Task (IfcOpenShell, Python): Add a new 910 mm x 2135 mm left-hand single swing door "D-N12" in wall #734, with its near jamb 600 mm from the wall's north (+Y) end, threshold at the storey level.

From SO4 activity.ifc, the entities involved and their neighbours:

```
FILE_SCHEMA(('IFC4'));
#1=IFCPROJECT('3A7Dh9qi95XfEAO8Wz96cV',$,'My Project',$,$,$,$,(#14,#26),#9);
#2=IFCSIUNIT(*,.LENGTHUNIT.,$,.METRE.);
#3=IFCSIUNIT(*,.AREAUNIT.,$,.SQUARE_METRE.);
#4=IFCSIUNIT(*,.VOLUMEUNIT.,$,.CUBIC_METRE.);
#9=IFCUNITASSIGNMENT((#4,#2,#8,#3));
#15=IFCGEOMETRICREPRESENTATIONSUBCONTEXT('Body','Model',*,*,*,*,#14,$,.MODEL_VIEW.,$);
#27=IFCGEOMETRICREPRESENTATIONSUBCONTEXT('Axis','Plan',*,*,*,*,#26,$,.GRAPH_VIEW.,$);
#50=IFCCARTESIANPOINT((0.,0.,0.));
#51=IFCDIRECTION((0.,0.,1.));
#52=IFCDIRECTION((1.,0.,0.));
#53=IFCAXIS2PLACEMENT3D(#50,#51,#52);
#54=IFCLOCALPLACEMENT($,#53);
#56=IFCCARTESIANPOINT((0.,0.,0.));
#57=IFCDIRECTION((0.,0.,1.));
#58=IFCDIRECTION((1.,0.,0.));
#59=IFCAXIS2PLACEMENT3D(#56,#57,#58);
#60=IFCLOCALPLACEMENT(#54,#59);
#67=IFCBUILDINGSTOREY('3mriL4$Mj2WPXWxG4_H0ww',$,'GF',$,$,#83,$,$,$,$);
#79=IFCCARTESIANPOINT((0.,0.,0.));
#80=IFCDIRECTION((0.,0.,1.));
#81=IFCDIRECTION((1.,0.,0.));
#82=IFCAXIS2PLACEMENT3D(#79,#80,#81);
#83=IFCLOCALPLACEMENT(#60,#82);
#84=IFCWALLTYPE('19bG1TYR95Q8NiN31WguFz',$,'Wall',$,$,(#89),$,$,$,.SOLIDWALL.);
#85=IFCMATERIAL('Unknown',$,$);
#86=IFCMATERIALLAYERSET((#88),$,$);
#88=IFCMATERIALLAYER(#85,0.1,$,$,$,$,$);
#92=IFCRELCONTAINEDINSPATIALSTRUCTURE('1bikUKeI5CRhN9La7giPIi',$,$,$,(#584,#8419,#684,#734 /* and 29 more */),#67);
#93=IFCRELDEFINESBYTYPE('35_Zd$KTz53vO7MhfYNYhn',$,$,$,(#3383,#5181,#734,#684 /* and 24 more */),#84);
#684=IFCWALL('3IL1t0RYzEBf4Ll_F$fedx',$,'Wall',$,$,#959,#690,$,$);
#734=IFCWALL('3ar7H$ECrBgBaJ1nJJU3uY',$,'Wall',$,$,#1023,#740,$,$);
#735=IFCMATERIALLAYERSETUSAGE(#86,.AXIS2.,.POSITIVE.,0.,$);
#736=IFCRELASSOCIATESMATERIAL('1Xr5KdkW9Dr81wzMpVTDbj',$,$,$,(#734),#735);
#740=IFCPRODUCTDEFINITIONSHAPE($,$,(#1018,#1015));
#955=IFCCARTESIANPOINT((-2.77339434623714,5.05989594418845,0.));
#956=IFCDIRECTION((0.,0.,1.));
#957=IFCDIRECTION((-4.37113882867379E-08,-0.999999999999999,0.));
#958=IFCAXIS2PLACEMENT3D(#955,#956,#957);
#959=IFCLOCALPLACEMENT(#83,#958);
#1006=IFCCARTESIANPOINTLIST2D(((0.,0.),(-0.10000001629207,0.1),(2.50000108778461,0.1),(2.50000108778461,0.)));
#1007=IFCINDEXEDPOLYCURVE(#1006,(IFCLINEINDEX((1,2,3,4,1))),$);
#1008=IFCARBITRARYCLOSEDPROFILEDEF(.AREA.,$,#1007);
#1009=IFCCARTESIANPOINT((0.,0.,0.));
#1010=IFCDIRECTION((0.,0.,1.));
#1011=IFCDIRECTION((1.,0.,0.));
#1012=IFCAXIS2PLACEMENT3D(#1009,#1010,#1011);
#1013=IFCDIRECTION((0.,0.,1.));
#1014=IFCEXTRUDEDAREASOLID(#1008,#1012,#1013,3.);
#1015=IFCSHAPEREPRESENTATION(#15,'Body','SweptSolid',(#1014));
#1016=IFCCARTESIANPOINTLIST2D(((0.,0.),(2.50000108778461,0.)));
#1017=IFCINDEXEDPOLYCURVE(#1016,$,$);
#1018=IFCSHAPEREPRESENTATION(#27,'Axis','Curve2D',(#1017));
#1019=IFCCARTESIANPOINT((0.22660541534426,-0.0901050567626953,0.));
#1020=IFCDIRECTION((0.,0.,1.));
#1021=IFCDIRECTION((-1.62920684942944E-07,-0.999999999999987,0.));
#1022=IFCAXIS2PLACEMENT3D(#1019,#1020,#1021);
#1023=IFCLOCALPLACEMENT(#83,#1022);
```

```python
import numpy as np
import ifcopenshell
import ifcopenshell.api.feature
import ifcopenshell.api.geometry
import ifcopenshell.api.root
import ifcopenshell.api.spatial
import ifcopenshell.geom
import ifcopenshell.util.element
import ifcopenshell.util.placement
import ifcopenshell.util.representation
import ifcopenshell.util.shape
import ifcopenshell.util.unit

model = ifcopenshell.open("SO4 activity.ifc")
unit_scale = ifcopenshell.util.unit.calculate_unit_scale(model)
settings = ifcopenshell.geom.settings()


def volume(element):
    """Net volume in cubic metres, openings subtracted."""
    shape = ifcopenshell.geom.create_shape(settings, element)
    return ifcopenshell.util.shape.get_volume(shape.geometry)


wall = model.by_guid("3ar7H$ECrBgBaJ1nJJU3uY")
storey = ifcopenshell.util.element.get_container(wall, ifc_class="IfcBuildingStorey")
context = ifcopenshell.util.representation.get_context(model, "Model", "Body", "MODEL_VIEW")
before = volume(wall)

width, height, from_end, sill = 0.91, 2.135, 0.6, 0.0  # metres

# The wall runs along its own X axis, and the end named is its -X end.
wall_shape = ifcopenshell.geom.create_shape(settings, wall)
x, y, z = ifcopenshell.util.shape.get_vertices(wall_shape.geometry).T
start = x.min() + from_end
face, thickness = float(y.min()), float(y.max() - y.min())
wall_matrix = ifcopenshell.util.placement.get_local_placement(wall.ObjectPlacement)
level = ifcopenshell.util.placement.get_local_placement(storey.ObjectPlacement)[2, 3]


def in_wall(x, y):
    """Placement at x, y metres in the wall's axes, at sill height."""
    matrix = wall_matrix.copy()
    matrix[:, 3] = wall_matrix @ np.array([x / unit_scale, y / unit_scale, 0.0, 1.0])
    matrix[2, 3] = level + sill / unit_scale
    return matrix


# Opening: a box that overshoots both wall faces by 50 mm.
opening = ifcopenshell.api.root.create_entity(model, ifc_class="IfcOpeningElement", predefined_type="OPENING")
box = ifcopenshell.api.geometry.add_wall_representation(
    model, context=context, length=width, height=height, thickness=thickness + 0.1
)
ifcopenshell.api.geometry.assign_representation(model, product=opening, representation=box)
ifcopenshell.api.geometry.edit_object_placement(model, product=opening, matrix=in_wall(start, face - 0.05), is_si=False)
ifcopenshell.api.feature.add_feature(model, feature=opening, element=wall)

door = ifcopenshell.api.root.create_entity(model, ifc_class="IfcDoor", name="D-N12", predefined_type="DOOR")
door.OverallWidth, door.OverallHeight = width / unit_scale, height / unit_scale
door.OperationType = "SINGLE_SWING_LEFT"
body = ifcopenshell.api.geometry.add_door_representation(
    model,
    context=context,
    overall_width=door.OverallWidth,
    overall_height=door.OverallHeight,
    operation_type="SINGLE_SWING_LEFT",
    lining_properties={"LiningDepth": thickness / unit_scale, "ThresholdDepth": thickness / unit_scale},
)
ifcopenshell.api.geometry.assign_representation(model, product=door, representation=body)
ifcopenshell.api.spatial.assign_container(model, products=[door], relating_structure=storey)
ifcopenshell.api.feature.add_filling(model, opening=opening, element=door)

# The lining spans the wall, so the door starts at the wall face.
ifcopenshell.api.geometry.edit_object_placement(model, product=door, matrix=in_wall(start, face), is_si=False)

after = volume(wall)

print(f"wall volume {before:.3f} -> {after:.3f} m3")

model.write("SO4 activity-out.ifc")
```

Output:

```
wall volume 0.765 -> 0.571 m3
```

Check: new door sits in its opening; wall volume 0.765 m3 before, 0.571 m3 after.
